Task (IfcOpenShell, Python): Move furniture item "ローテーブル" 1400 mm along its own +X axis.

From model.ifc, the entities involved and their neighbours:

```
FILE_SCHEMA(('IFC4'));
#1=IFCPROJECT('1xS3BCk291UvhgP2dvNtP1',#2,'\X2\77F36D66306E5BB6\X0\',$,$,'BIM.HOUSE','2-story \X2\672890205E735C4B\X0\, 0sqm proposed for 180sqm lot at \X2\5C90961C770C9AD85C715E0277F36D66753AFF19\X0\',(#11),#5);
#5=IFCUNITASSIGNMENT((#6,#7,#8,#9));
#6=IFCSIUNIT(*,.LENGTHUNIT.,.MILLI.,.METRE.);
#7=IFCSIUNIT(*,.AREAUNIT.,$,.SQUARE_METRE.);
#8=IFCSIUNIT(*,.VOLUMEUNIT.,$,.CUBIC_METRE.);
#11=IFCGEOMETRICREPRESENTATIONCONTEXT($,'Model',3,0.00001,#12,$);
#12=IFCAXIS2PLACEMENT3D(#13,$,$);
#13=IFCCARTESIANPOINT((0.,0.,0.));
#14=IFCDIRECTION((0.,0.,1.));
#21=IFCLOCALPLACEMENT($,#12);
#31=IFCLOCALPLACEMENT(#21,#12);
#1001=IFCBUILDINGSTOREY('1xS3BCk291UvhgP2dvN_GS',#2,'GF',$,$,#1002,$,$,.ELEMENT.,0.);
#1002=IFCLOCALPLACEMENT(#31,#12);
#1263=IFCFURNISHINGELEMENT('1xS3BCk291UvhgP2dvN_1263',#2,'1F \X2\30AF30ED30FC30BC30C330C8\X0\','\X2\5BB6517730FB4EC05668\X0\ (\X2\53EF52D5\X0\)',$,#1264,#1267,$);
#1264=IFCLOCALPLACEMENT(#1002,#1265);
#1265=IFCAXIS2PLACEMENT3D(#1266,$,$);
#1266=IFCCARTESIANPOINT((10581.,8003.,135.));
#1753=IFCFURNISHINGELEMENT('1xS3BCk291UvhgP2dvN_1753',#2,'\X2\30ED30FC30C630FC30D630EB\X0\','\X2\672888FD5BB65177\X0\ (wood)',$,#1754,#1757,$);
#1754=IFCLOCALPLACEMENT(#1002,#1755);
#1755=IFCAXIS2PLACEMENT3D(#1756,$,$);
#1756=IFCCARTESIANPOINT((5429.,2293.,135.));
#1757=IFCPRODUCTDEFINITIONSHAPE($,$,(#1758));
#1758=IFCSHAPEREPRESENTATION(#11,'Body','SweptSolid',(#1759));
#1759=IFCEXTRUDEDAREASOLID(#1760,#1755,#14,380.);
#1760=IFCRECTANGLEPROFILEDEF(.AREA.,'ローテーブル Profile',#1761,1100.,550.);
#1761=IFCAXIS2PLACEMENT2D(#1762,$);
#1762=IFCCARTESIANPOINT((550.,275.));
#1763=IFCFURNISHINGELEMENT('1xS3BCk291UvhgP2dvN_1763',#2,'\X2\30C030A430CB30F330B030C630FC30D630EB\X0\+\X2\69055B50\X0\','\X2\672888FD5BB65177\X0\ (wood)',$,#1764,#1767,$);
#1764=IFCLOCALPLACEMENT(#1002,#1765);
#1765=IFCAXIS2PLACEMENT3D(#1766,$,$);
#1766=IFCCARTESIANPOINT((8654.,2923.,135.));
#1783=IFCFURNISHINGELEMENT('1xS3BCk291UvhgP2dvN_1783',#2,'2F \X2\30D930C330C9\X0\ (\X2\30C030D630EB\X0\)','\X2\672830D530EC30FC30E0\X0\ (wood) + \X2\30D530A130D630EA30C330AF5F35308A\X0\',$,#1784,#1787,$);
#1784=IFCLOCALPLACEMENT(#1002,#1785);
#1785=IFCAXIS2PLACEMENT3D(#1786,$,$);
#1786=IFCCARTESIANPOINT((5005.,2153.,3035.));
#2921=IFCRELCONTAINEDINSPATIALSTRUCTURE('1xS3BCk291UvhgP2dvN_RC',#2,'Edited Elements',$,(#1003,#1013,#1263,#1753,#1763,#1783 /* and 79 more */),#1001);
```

```python
import ifcopenshell
import ifcopenshell.api.geometry
import ifcopenshell.util.placement

model = ifcopenshell.open("model.ifc")

item = model.by_guid("1xS3BCk291UvhgP2dvN_1753")
matrix = ifcopenshell.util.placement.get_local_placement(item.ObjectPlacement)
matrix[:3, 3] += matrix[:3, 0] * 1400.0
ifcopenshell.api.geometry.edit_object_placement(model, product=item, matrix=matrix, is_si=False)

print(ifcopenshell.util.placement.get_local_placement(item.ObjectPlacement).round(3) + 0.0)

model.write("model_rev.ifc")
```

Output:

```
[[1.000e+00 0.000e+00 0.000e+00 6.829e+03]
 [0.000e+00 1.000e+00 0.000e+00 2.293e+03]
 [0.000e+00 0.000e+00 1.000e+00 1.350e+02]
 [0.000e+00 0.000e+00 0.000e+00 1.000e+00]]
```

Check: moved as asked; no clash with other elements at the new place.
